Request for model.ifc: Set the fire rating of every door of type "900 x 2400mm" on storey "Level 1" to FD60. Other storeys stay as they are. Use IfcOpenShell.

First a look at what the model holds.

```python
import ifcopenshell
import ifcopenshell.util.element

model = ifcopenshell.open("model.ifc")
print(model.schema)
storey = next(s for s in model.by_type("IfcBuildingStorey") if s.Name == "Level 1")
doors = [e for e in ifcopenshell.util.element.get_decomposition(storey) if e.is_a("IfcDoor")]
seen = {}
for e in doors:
    element_type = ifcopenshell.util.element.get_type(e)
    key = (element_type.Name if element_type != e and element_type else None, ifcopenshell.util.element.get_pset(e, "Pset_DoorCommon", "FireRating"))
    seen[key] = seen.get(key, 0) + 1
for (name, value), count in sorted(seen.items(), key=str):
    print(count, "x", name, "|", value)
```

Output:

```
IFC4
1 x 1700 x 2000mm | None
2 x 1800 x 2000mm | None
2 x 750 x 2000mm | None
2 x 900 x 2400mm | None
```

```python
import ifcopenshell
import ifcopenshell.api.pset
import ifcopenshell.util.element

model = ifcopenshell.open("model.ifc")

storey = next(s for s in model.by_type("IfcBuildingStorey") if s.Name == "Level 1")
doors = [e for e in ifcopenshell.util.element.get_decomposition(storey) if e.is_a("IfcDoor")]

count = 0
for e in doors:
    element_type = ifcopenshell.util.element.get_type(e)
    if element_type in (None, e) or element_type.Name != "900 x 2400mm":
        continue
    # add_pset returns the element's existing set when there is one.
    pset = ifcopenshell.api.pset.add_pset(model, product=e, name="Pset_DoorCommon")
    ifcopenshell.api.pset.edit_pset(model, pset=pset, properties={"FireRating": "FD60"})
    count += 1

print(count, "doors updated")

model.write("model_edited.ifc")
```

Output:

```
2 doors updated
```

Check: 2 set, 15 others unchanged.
